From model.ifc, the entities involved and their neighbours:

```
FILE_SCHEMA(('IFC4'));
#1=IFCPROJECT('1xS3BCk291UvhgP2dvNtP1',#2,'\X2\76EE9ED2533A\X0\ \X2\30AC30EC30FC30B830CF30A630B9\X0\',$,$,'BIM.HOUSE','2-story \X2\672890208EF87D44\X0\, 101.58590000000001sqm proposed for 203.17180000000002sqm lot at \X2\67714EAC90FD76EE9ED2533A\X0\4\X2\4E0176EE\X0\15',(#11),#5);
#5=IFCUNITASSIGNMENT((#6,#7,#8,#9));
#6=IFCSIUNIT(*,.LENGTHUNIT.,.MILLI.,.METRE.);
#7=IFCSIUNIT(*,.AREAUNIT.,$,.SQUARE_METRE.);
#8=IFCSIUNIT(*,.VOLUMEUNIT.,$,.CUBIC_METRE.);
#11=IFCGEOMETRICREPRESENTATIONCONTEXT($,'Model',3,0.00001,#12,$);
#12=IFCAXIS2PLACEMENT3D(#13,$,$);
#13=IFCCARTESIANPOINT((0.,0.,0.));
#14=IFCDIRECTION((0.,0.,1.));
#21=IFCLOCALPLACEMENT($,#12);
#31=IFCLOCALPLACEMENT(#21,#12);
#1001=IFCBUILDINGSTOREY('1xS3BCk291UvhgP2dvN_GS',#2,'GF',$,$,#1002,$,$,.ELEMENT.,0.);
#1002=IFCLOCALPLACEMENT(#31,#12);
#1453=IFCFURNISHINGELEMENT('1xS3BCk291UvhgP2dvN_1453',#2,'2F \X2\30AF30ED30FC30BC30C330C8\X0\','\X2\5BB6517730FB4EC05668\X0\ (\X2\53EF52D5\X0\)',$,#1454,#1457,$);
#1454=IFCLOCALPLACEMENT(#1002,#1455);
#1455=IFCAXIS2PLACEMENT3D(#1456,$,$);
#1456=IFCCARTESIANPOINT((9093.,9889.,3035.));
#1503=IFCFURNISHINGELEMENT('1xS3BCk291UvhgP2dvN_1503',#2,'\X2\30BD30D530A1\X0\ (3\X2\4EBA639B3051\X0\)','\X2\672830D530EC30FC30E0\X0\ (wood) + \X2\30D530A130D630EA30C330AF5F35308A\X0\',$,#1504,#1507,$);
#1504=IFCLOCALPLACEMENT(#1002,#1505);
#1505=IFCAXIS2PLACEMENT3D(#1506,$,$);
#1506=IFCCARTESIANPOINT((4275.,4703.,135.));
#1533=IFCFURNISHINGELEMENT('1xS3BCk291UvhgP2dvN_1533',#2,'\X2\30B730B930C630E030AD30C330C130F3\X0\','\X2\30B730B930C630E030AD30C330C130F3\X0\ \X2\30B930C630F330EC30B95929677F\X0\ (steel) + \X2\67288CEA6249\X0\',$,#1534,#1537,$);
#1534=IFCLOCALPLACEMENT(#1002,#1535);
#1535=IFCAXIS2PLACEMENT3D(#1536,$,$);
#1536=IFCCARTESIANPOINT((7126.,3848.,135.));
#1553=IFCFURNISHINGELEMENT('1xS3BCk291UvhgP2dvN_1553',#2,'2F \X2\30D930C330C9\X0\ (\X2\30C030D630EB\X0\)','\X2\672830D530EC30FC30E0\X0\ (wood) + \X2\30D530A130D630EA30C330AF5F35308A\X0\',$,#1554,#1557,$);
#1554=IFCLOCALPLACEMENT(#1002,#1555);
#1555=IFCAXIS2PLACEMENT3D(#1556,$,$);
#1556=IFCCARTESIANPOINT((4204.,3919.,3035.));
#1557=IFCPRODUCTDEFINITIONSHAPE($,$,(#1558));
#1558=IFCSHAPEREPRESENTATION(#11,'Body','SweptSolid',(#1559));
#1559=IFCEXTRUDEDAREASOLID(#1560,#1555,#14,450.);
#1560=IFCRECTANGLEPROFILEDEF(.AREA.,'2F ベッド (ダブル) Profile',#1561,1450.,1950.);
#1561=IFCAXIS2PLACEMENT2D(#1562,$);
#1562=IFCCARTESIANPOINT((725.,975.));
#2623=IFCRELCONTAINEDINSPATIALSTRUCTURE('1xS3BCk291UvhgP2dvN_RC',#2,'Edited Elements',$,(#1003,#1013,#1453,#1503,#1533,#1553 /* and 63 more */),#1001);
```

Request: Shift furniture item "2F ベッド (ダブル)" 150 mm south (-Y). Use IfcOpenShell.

```python
import ifcopenshell
import ifcopenshell.api.geometry
import ifcopenshell.util.placement
import ifcopenshell.util.unit

model = ifcopenshell.open("model.ifc")
unit_scale = ifcopenshell.util.unit.calculate_unit_scale(model)

item = model.by_guid("1xS3BCk291UvhgP2dvN_1553")
matrix = ifcopenshell.util.placement.get_local_placement(item.ObjectPlacement)
matrix[1, 3] -= 0.15 / unit_scale
ifcopenshell.api.geometry.edit_object_placement(model, product=item, matrix=matrix, is_si=False)

print(ifcopenshell.util.placement.get_local_placement(item.ObjectPlacement).round(3) + 0.0)

model.write("model_v2.ifc")
```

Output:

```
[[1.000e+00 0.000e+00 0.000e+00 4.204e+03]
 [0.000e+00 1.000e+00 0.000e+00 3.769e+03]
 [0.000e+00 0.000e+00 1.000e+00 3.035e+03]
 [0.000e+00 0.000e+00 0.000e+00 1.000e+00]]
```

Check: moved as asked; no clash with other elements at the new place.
